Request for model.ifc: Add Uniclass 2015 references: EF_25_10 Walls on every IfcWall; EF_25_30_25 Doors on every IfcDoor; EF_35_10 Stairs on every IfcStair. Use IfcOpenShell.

First a look at what the model holds.

```python
import ifcopenshell

model = ifcopenshell.open("model.ifc")
print(model.schema)
print("classifications:", [c.Name for c in model.by_type("IfcClassification")])
for ifc_class in ("IfcDoor", "IfcRoof", "IfcStair", "IfcWall", "IfcWindow"):
    print(ifc_class, len(model.by_type(ifc_class)))
```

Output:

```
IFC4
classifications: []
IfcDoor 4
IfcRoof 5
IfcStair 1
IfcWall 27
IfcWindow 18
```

```python
import ifcopenshell
import ifcopenshell.api.classification

model = ifcopenshell.open("model.ifc")

system = ifcopenshell.api.classification.add_classification(model, classification="Uniclass 2015")

codes = {
    "IfcWall": ("EF_25_10", "Walls"),
    "IfcDoor": ("EF_25_30_25", "Doors"),
    "IfcStair": ("EF_35_10", "Stairs"),
}
for ifc_class, (code, name) in codes.items():
    products = model.by_type(ifc_class)
    ifcopenshell.api.classification.add_reference(
        model, products=products, classification=system, identification=code, name=name
    )
    print(code, len(products))

model.write("model-out.ifc")
```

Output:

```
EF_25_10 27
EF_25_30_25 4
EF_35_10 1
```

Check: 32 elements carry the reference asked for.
